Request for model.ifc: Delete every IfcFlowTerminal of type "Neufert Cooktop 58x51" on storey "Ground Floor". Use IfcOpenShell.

First a look at what the model holds.

```python
import ifcopenshell
import ifcopenshell.util.element

model = ifcopenshell.open("model.ifc")
print(model.schema)
storey = next(s for s in model.by_type("IfcBuildingStorey") if s.Name == "Ground Floor")
terminals = [e for e in ifcopenshell.util.element.get_decomposition(storey) if e.is_a("IfcFlowTerminal")]
seen = {}
for e in terminals:
    element_type = ifcopenshell.util.element.get_type(e)
    name = element_type.Name if element_type not in (None, e) else None
    seen[name] = seen.get(name, 0) + 1
for name, count in sorted(seen.items(), key=str):
    print(count, "x", name)
```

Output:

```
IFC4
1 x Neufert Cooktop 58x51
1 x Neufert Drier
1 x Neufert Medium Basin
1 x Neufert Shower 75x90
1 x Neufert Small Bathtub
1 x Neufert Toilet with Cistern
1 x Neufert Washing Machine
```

```python
import ifcopenshell
import ifcopenshell.api.root
import ifcopenshell.util.element

model = ifcopenshell.open("model.ifc")

storey = next(s for s in model.by_type("IfcBuildingStorey") if s.Name == "Ground Floor")
terminals = [e for e in ifcopenshell.util.element.get_decomposition(storey) if e.is_a("IfcFlowTerminal")]
targets = [e for e in terminals if (t := ifcopenshell.util.element.get_type(e)) not in (None, e) and t.Name == "Neufert Cooktop 58x51"]

for e in targets:
    ifcopenshell.api.root.remove_product(model, product=e)
print(len(targets), "removed")

model.write("model_v2.ifc")
```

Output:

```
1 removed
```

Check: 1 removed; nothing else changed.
